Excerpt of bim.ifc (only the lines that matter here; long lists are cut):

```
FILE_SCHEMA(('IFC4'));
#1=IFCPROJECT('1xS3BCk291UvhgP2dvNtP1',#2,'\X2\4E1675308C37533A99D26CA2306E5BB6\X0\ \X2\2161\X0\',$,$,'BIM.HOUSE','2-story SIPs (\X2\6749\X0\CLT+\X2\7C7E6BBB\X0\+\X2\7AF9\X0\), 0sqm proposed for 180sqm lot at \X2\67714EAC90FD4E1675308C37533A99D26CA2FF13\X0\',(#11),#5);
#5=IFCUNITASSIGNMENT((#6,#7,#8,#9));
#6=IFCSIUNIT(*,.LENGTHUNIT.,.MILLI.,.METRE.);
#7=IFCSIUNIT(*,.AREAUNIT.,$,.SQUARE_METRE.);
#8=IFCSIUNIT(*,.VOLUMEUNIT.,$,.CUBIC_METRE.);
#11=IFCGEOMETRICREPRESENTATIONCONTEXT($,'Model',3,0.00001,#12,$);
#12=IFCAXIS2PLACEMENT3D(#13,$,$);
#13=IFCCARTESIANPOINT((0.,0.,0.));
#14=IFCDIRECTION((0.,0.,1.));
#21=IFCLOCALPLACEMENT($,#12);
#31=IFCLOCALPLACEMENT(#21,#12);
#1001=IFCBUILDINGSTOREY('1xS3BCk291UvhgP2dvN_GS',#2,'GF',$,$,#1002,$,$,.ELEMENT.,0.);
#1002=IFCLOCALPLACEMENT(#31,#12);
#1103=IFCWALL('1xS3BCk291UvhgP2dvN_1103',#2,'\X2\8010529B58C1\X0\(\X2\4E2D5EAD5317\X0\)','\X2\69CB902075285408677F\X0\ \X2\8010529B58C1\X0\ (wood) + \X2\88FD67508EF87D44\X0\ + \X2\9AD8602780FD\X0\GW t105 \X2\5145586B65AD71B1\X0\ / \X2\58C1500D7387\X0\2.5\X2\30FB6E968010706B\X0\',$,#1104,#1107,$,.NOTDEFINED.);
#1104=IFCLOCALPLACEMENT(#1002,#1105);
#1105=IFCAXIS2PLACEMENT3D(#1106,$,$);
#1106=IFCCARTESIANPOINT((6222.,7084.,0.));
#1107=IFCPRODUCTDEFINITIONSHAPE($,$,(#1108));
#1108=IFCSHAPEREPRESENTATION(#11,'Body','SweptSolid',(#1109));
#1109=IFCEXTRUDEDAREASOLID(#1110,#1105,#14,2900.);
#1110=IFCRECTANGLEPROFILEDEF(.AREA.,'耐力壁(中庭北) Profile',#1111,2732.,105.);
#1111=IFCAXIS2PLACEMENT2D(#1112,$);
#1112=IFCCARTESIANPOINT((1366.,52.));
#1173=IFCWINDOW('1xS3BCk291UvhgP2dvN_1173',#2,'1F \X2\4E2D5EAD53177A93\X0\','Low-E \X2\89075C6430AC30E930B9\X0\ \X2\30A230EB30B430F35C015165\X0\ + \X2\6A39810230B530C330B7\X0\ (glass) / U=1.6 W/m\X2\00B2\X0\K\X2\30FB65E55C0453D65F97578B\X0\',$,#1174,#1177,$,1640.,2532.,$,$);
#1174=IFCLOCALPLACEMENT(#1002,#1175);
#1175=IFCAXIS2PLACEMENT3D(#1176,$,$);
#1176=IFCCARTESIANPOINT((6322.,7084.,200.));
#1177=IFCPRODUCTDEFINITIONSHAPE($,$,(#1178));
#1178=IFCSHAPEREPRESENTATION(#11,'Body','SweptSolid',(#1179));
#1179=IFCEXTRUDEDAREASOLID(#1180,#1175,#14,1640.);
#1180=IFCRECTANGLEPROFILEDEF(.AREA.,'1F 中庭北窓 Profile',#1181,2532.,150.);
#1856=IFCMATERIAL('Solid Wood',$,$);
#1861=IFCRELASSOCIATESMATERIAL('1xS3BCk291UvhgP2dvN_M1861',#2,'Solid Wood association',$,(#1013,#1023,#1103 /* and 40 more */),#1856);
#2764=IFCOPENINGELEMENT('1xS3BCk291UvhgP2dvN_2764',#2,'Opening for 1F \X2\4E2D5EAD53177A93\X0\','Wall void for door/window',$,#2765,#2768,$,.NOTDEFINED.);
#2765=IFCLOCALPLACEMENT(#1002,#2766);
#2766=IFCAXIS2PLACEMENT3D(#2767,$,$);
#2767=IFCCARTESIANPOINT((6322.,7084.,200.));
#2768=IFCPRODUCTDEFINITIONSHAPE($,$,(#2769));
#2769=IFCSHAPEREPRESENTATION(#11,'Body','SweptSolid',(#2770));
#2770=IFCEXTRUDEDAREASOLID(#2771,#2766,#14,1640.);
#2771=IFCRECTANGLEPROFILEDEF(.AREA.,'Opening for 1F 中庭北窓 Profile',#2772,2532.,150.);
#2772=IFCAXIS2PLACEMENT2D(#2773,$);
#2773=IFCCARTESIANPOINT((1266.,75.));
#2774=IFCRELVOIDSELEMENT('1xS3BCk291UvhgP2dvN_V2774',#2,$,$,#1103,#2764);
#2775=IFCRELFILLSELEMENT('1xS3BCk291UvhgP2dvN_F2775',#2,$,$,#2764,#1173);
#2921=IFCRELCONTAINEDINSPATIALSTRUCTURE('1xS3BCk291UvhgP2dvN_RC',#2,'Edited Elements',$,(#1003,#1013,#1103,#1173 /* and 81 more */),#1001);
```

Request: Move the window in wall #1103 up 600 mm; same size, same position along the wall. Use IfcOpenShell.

```python
import numpy as np
import ifcopenshell
import ifcopenshell.api.geometry
import ifcopenshell.util.placement
import ifcopenshell.util.unit

model = ifcopenshell.open("bim.ifc")
unit_scale = ifcopenshell.util.unit.calculate_unit_scale(model)

window = model.by_guid("1xS3BCk291UvhgP2dvN_1173")
opening = window.FillsVoids[0].RelatingOpeningElement
dz = 0.6 / unit_scale

shift = np.array([0.0, 0.0, dz])
# The window is not placed relative to its opening, so move both.
for product in (opening, window):
    matrix = ifcopenshell.util.placement.get_local_placement(product.ObjectPlacement)
    matrix[:3, 3] += shift
    ifcopenshell.api.geometry.edit_object_placement(model, product=product, matrix=matrix, is_si=False)

print(f"moved by {dz * unit_scale:+.3f} m")

model.write("bim_edited.ifc")
```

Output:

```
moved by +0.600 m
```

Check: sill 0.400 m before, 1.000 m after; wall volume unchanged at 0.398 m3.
